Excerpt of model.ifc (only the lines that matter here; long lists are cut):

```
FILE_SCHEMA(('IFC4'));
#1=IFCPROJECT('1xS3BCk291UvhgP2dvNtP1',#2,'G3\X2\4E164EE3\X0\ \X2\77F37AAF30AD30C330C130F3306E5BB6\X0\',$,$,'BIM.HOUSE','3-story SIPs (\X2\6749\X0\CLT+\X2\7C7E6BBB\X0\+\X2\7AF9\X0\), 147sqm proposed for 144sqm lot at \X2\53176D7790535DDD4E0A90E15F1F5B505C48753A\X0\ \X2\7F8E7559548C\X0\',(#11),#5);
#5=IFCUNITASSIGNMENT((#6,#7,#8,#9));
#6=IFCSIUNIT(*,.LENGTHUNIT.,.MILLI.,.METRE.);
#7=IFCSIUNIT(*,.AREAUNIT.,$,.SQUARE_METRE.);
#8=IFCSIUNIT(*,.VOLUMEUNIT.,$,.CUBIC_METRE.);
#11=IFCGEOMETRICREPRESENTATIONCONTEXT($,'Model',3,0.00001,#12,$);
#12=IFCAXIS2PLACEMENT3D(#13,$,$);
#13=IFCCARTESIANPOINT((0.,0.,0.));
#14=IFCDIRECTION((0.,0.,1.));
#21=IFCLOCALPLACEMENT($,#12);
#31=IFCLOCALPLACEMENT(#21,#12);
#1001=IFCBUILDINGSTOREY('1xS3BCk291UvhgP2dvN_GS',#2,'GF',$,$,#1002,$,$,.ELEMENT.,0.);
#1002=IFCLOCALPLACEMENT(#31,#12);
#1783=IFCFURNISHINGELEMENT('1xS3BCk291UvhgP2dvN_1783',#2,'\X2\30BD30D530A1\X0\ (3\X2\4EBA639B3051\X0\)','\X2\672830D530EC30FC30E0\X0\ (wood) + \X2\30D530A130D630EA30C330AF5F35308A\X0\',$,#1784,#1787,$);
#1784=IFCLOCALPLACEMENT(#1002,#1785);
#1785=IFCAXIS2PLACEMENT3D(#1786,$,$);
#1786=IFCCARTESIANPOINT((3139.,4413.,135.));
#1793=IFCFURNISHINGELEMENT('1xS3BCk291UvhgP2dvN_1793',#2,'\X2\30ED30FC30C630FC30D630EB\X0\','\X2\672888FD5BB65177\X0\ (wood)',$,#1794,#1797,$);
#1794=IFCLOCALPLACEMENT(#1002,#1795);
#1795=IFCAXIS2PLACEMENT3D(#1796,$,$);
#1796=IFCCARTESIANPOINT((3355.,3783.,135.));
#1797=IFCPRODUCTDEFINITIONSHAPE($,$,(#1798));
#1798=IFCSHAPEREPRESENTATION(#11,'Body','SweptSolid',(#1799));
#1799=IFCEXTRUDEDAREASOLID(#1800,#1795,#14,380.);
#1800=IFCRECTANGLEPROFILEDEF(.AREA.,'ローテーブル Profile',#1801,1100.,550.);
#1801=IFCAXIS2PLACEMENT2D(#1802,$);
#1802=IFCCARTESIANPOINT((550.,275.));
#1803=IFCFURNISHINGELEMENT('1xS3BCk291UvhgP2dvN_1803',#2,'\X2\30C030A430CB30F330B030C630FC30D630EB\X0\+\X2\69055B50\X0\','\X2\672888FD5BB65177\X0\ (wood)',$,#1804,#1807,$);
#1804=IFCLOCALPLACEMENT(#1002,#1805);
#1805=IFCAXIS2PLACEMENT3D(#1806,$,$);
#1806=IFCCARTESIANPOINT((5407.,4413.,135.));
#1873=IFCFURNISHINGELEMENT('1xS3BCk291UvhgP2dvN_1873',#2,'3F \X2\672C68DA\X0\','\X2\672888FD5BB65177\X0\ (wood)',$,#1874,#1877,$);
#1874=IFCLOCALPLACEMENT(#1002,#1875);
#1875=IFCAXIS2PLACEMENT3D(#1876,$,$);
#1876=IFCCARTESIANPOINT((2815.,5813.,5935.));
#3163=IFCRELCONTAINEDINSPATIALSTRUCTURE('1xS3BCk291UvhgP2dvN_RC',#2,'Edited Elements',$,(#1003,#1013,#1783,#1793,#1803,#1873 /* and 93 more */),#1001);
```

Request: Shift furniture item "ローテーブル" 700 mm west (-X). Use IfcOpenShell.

```python
import ifcopenshell
import ifcopenshell.api.geometry
import ifcopenshell.util.placement
import ifcopenshell.util.unit

model = ifcopenshell.open("model.ifc")
unit_scale = ifcopenshell.util.unit.calculate_unit_scale(model)

item = model.by_guid("1xS3BCk291UvhgP2dvN_1793")
matrix = ifcopenshell.util.placement.get_local_placement(item.ObjectPlacement)
matrix[0, 3] -= 0.7 / unit_scale
ifcopenshell.api.geometry.edit_object_placement(model, product=item, matrix=matrix, is_si=False)

print(ifcopenshell.util.placement.get_local_placement(item.ObjectPlacement).round(3) + 0.0)

model.write("model_updated.ifc")
```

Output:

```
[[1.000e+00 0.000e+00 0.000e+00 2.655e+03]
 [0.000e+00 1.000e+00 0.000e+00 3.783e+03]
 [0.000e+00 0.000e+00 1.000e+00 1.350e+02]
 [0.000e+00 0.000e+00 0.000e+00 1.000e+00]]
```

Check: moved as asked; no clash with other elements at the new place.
